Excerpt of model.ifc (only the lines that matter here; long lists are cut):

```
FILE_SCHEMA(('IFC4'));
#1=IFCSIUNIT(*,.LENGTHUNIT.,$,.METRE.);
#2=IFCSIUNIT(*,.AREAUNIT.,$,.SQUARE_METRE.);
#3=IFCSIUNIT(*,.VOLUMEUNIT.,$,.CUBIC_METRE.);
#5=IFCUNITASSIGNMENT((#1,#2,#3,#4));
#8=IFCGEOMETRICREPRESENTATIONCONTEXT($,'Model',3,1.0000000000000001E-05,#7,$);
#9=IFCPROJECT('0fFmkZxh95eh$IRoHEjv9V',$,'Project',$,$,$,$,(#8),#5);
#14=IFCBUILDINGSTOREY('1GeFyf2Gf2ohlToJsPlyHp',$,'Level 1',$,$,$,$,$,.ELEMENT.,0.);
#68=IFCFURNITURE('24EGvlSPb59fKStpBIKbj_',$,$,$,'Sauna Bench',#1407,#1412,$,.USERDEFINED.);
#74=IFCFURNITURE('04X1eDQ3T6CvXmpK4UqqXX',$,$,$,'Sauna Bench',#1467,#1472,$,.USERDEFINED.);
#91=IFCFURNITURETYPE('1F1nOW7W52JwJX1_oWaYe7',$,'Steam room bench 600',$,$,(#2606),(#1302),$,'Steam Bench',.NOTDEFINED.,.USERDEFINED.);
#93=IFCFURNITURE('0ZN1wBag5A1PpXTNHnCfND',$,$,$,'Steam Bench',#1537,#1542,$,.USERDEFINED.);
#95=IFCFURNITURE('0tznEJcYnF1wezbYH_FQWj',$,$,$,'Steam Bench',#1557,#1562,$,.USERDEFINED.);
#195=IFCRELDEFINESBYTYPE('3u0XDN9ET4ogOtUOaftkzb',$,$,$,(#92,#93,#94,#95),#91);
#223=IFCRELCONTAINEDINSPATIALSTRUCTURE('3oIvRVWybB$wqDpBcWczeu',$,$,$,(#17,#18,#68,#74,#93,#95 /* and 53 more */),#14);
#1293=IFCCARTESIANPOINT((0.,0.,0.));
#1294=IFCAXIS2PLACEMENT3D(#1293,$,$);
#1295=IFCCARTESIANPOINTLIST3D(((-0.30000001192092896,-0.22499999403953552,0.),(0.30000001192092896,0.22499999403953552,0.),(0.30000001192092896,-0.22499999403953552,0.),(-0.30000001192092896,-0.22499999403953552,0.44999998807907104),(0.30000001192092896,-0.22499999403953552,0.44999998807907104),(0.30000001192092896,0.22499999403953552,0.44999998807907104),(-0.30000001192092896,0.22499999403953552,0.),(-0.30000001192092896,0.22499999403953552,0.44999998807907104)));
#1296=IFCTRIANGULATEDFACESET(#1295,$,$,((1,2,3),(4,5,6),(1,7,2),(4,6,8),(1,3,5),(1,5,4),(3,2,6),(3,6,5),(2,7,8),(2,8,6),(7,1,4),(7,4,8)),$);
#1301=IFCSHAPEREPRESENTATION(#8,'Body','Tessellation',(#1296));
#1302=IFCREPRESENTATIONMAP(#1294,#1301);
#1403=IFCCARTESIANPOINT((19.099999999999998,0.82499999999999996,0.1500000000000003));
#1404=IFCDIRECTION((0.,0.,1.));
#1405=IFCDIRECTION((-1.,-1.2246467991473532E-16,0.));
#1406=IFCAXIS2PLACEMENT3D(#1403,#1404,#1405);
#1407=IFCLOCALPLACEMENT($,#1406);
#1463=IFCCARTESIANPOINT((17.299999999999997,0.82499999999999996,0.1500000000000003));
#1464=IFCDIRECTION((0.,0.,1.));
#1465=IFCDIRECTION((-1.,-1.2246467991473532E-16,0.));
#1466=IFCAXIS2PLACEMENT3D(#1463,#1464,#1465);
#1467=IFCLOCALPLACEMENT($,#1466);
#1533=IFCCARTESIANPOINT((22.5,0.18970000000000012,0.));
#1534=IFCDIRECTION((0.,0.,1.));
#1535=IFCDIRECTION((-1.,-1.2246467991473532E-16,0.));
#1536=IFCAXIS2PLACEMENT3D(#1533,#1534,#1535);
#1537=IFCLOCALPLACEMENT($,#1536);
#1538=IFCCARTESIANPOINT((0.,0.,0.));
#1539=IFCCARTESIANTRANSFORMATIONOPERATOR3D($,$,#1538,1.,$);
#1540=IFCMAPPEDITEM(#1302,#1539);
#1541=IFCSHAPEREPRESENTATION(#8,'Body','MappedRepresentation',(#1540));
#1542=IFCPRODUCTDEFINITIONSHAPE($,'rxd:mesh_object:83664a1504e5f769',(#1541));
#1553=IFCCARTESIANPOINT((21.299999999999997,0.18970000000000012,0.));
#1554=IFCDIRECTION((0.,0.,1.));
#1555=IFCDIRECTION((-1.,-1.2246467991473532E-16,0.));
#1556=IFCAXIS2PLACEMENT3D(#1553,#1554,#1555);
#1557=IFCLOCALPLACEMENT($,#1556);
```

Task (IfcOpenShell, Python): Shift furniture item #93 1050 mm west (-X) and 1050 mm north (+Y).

```python
import ifcopenshell
import ifcopenshell.api.geometry
import ifcopenshell.util.placement
import ifcopenshell.util.unit

model = ifcopenshell.open("model.ifc")
unit_scale = ifcopenshell.util.unit.calculate_unit_scale(model)

item = model.by_guid("0ZN1wBag5A1PpXTNHnCfND")
matrix = ifcopenshell.util.placement.get_local_placement(item.ObjectPlacement)
matrix[0, 3] -= 1.05 / unit_scale
matrix[1, 3] += 1.05 / unit_scale
ifcopenshell.api.geometry.edit_object_placement(model, product=item, matrix=matrix, is_si=False)

print(ifcopenshell.util.placement.get_local_placement(item.ObjectPlacement).round(3) + 0.0)

model.write("model_edited.ifc")
```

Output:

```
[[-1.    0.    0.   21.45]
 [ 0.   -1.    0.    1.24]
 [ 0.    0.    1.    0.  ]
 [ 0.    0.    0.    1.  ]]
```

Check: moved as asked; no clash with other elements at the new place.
